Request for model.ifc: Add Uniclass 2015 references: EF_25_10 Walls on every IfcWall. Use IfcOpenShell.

First a look at what the model holds.

```python
import ifcopenshell

model = ifcopenshell.open("model.ifc")
print(model.schema)
print("classifications:", [c.Name for c in model.by_type("IfcClassification")])
for ifc_class in ("IfcDoor", "IfcRoof", "IfcStair", "IfcWall", "IfcWindow"):
    print(ifc_class, len(model.by_type(ifc_class)))
```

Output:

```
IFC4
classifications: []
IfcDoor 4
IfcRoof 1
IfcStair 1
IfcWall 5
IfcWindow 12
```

```python
import ifcopenshell
import ifcopenshell.api.classification

model = ifcopenshell.open("model.ifc")

system = ifcopenshell.api.classification.add_classification(model, classification="Uniclass 2015")

codes = {
    "IfcWall": ("EF_25_10", "Walls"),
}
for ifc_class, (code, name) in codes.items():
    products = model.by_type(ifc_class)
    ifcopenshell.api.classification.add_reference(
        model, products=products, classification=system, identification=code, name=name
    )
    print(code, len(products))

model.write("model_v2.ifc")
```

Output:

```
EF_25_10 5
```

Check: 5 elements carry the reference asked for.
